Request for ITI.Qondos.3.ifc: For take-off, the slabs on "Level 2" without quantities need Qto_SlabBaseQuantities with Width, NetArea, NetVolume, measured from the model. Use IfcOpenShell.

First a look at what the model holds.

```python
import ifcopenshell
import ifcopenshell.util.element
import ifcopenshell.util.unit

model = ifcopenshell.open("ITI.Qondos.3.ifc")
print(model.schema)
for unit_type in ("LENGTHUNIT", "AREAUNIT", "VOLUMEUNIT"):
    print(unit_type, ifcopenshell.util.unit.calculate_unit_scale(model, unit_type))
storey = next(s for s in model.by_type("IfcBuildingStorey") if s.Name == "Level 2")
slabs = [e for e in ifcopenshell.util.element.get_decomposition(storey) if e.is_a("IfcSlab")]
for e in sorted(slabs, key=lambda e: e.id()):
    print(e.id(), e.is_a(), e.Name, list(ifcopenshell.util.element.get_psets(e, qtos_only=True)), sep=" | ")
```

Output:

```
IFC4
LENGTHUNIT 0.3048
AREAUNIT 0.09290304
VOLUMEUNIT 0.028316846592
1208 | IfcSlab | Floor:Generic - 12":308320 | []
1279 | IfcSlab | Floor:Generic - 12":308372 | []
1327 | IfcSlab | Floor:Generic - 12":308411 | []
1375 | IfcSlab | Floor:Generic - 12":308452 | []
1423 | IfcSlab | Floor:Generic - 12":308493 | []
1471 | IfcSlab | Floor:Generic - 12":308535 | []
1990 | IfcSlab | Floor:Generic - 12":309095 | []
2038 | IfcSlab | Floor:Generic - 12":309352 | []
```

```python
import ifcopenshell
import ifcopenshell.api.pset
import ifcopenshell.geom
import ifcopenshell.util.element
import ifcopenshell.util.shape
import ifcopenshell.util.unit

model = ifcopenshell.open("ITI.Qondos.3.ifc")
unit_scale = ifcopenshell.util.unit.calculate_unit_scale(model)
area_scale = ifcopenshell.util.unit.calculate_unit_scale(model, "AREAUNIT")
volume_scale = ifcopenshell.util.unit.calculate_unit_scale(model, "VOLUMEUNIT")
settings = ifcopenshell.geom.settings()

storey = next(s for s in model.by_type("IfcBuildingStorey") if s.Name == "Level 2")
slabs = [e for e in ifcopenshell.util.element.get_decomposition(storey) if e.is_a("IfcSlab")]

for e in sorted(slabs, key=lambda e: e.id()):
    if ifcopenshell.util.element.get_psets(e, qtos_only=True, should_inherit=False):
        continue
    # Geometry comes back in metres, in the element's own axes.
    shape = ifcopenshell.geom.create_shape(settings, e)
    values = {
        "Width": ifcopenshell.util.shape.get_z(shape.geometry) / unit_scale,
        "NetArea": ifcopenshell.util.shape.get_footprint_area(shape.geometry) / area_scale,
        "NetVolume": ifcopenshell.util.shape.get_volume(shape.geometry) / volume_scale,
    }
    qto = ifcopenshell.api.pset.add_qto(model, product=e, name="Qto_SlabBaseQuantities")
    ifcopenshell.api.pset.edit_qto(model, qto=qto, properties=values)
    print(e.id(), {k: round(v, 3) for k, v in values.items()})

model.write("ITI.Qondos.3_v2.ifc")
```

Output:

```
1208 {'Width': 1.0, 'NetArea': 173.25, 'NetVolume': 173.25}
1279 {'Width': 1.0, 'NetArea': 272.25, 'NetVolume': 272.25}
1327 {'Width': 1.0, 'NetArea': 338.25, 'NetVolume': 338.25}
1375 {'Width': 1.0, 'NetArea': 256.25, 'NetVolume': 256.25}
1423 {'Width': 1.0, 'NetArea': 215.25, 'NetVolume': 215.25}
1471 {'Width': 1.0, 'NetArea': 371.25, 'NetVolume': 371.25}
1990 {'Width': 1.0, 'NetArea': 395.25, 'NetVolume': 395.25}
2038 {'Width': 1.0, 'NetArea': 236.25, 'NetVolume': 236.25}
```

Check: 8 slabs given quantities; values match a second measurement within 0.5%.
